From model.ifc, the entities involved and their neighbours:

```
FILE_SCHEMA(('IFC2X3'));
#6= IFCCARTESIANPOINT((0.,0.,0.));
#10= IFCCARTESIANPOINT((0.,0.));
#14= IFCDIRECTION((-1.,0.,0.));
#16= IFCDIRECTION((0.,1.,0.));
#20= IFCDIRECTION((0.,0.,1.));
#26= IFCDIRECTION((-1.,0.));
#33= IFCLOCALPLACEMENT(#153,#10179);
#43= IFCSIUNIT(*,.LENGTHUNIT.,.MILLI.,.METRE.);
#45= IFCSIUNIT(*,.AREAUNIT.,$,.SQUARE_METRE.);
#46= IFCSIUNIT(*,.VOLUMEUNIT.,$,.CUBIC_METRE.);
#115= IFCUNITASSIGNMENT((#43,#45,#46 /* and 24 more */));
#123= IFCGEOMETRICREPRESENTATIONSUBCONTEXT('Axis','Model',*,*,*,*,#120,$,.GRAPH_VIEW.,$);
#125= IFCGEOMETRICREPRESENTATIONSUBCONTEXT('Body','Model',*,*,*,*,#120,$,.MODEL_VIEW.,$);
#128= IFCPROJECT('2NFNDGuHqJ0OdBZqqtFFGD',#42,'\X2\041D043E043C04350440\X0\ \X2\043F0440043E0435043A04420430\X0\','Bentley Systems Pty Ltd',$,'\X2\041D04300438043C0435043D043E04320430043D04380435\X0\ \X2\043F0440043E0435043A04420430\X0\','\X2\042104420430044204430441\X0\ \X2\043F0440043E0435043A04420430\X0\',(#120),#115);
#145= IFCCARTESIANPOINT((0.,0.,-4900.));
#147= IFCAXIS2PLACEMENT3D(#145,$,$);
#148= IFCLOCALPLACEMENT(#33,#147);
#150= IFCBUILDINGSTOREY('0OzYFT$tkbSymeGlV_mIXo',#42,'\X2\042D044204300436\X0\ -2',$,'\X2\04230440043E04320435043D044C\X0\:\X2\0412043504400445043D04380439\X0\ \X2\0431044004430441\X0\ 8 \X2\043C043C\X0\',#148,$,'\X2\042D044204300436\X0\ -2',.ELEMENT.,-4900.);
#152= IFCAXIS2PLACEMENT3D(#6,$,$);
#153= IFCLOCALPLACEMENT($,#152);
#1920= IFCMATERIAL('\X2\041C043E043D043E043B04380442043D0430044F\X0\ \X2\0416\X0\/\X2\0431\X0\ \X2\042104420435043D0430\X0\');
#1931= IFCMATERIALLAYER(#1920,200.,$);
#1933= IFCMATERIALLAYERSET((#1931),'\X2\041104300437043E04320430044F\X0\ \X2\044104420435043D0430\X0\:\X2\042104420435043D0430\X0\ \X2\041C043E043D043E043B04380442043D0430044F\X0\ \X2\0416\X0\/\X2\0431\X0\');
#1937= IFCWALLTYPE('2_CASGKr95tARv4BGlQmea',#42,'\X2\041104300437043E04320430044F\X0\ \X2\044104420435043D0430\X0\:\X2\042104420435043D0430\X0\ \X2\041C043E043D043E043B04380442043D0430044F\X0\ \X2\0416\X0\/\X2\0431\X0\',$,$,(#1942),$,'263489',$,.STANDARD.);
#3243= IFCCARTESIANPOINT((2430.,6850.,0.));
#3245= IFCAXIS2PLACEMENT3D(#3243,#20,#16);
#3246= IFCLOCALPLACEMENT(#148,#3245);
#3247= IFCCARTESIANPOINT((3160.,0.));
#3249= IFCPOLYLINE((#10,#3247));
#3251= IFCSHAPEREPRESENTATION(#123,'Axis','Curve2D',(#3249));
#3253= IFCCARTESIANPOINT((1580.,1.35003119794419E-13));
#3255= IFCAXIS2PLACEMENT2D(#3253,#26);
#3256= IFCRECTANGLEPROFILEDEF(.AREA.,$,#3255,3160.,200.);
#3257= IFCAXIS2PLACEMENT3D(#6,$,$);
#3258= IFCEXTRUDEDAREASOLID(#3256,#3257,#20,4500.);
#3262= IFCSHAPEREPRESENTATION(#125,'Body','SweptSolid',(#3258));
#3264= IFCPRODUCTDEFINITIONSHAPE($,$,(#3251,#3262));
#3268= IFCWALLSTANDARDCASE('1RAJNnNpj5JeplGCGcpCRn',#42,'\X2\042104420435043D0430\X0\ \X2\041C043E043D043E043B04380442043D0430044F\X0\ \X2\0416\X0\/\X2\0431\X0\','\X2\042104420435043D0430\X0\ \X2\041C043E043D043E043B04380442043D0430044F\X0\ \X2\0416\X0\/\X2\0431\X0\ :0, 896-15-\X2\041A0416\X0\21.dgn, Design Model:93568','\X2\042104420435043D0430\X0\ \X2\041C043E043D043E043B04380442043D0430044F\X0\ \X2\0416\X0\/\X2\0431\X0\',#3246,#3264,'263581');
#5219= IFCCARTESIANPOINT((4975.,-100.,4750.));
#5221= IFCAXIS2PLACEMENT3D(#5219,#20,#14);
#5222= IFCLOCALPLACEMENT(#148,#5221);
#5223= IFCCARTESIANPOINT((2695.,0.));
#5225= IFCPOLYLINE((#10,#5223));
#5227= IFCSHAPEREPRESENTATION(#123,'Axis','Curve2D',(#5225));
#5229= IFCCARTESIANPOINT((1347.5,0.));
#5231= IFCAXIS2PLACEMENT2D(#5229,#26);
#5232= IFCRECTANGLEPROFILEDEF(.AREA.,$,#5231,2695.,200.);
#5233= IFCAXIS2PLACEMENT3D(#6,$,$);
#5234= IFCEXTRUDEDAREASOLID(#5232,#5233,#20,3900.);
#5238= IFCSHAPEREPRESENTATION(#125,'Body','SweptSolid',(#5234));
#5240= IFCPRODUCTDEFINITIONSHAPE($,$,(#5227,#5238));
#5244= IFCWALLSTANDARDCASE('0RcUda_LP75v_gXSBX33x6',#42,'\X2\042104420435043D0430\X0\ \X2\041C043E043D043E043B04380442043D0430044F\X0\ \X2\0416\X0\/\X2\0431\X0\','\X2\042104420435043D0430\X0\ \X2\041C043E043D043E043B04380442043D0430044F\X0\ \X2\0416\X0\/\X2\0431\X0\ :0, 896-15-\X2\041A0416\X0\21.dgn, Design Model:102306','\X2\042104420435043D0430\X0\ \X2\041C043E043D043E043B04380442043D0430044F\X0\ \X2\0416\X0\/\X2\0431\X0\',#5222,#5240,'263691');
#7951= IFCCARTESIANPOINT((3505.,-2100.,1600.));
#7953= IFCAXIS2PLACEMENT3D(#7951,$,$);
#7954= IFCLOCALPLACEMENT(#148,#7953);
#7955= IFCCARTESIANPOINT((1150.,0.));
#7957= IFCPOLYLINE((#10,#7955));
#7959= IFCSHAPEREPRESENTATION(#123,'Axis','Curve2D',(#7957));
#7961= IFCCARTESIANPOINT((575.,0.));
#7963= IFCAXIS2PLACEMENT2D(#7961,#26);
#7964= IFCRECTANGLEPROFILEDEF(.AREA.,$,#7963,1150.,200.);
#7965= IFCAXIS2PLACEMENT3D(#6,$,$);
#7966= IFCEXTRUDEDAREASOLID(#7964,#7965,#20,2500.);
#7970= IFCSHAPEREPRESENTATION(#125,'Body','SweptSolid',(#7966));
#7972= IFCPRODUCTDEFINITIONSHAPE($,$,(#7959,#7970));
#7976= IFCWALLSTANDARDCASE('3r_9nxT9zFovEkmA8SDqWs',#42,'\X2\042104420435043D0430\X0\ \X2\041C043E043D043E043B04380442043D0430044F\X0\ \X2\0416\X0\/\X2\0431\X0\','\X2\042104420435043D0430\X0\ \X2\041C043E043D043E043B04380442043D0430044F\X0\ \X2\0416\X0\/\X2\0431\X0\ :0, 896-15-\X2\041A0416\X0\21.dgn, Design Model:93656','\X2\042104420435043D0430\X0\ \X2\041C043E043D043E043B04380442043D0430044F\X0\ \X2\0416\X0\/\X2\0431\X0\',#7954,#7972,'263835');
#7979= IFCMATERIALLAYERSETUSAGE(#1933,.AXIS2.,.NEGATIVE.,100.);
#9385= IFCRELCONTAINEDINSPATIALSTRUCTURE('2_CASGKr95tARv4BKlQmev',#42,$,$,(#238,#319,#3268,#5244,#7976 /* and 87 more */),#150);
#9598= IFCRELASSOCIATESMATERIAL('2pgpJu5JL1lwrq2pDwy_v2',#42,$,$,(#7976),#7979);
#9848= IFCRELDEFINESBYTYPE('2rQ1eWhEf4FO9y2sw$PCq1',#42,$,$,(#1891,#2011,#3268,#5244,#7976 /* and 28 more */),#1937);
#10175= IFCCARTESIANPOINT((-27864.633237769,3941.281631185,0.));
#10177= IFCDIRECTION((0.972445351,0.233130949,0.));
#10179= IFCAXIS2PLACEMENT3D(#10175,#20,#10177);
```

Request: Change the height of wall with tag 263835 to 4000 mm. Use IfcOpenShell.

```python
import ifcopenshell
import ifcopenshell.geom
import ifcopenshell.util.representation
import ifcopenshell.util.shape
import ifcopenshell.util.unit

model = ifcopenshell.open("model.ifc")
unit_scale = ifcopenshell.util.unit.calculate_unit_scale(model)
settings = ifcopenshell.geom.settings()


def volume(element):
    """Net volume in cubic metres, openings subtracted."""
    shape = ifcopenshell.geom.create_shape(settings, element)
    return ifcopenshell.util.shape.get_volume(shape.geometry)


wall = model.by_guid("3r_9nxT9zFovEkmA8SDqWs")
before = volume(wall)

body = ifcopenshell.util.representation.get_representation(wall, "Model", "Body")
solid = body.Items[0]
old_height = solid.Depth
solid.Depth = 4 / unit_scale
after = volume(wall)

print(f"height {old_height:g} -> {solid.Depth:g}, volume {before:.3f} -> {after:.3f} m3")

model.write("model_updated.ifc")
```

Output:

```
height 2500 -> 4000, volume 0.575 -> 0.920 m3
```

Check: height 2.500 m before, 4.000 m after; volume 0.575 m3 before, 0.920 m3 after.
